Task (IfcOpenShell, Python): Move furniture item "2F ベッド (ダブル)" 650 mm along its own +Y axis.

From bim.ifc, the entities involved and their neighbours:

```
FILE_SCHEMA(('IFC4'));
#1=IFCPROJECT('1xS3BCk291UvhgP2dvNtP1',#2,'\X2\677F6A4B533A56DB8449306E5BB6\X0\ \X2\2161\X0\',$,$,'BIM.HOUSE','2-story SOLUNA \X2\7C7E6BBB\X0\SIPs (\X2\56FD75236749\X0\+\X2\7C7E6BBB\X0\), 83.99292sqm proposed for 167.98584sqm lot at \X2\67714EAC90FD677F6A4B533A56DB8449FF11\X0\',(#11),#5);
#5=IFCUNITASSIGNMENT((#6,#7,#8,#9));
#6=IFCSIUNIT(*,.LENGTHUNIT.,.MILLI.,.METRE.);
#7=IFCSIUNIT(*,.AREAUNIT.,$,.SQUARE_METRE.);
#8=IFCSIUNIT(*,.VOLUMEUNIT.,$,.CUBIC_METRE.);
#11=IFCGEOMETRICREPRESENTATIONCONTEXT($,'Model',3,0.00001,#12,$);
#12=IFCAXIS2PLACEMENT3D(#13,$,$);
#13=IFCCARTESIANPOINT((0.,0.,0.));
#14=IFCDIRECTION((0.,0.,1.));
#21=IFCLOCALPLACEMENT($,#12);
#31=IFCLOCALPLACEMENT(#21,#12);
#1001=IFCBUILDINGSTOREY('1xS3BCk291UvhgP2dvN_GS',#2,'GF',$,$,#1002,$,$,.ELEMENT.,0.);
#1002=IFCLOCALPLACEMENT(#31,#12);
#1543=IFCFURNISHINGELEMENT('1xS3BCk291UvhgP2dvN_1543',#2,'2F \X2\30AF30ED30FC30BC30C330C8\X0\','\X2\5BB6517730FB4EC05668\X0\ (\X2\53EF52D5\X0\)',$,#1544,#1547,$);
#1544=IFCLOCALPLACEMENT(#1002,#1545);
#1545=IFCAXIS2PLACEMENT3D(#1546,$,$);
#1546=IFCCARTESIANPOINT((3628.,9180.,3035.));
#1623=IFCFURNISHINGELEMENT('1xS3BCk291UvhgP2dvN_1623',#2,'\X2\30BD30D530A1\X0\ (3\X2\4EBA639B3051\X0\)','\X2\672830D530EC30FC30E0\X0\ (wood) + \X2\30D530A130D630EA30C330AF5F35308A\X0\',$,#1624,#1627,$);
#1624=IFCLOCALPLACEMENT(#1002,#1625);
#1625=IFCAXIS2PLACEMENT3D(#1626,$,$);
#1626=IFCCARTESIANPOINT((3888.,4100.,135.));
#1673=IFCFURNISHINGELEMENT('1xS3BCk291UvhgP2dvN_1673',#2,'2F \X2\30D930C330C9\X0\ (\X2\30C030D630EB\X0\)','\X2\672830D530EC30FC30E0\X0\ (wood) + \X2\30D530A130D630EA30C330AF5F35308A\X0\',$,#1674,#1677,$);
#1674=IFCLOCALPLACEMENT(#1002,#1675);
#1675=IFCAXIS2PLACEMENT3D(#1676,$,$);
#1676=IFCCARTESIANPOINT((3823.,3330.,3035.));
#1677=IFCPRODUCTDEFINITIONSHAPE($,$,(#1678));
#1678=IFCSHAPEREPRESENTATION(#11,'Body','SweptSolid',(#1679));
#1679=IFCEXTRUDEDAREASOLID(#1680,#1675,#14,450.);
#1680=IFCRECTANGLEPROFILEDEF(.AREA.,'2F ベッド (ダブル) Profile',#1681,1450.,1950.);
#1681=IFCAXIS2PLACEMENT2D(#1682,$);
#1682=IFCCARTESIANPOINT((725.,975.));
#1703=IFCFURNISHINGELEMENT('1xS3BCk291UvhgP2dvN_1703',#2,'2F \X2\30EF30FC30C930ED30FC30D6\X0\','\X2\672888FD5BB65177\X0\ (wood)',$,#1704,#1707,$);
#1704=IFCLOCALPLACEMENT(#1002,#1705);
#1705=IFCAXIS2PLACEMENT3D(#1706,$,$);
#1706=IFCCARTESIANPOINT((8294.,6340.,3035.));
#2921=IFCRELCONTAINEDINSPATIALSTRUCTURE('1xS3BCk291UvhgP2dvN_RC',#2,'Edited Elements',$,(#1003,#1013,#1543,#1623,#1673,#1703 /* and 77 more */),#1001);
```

```python
import ifcopenshell
import ifcopenshell.api.geometry
import ifcopenshell.util.placement

model = ifcopenshell.open("bim.ifc")

item = model.by_guid("1xS3BCk291UvhgP2dvN_1673")
matrix = ifcopenshell.util.placement.get_local_placement(item.ObjectPlacement)
matrix[:3, 3] += matrix[:3, 1] * 650.0
ifcopenshell.api.geometry.edit_object_placement(model, product=item, matrix=matrix, is_si=False)

print(ifcopenshell.util.placement.get_local_placement(item.ObjectPlacement).round(3) + 0.0)

model.write("bim_v2.ifc")
```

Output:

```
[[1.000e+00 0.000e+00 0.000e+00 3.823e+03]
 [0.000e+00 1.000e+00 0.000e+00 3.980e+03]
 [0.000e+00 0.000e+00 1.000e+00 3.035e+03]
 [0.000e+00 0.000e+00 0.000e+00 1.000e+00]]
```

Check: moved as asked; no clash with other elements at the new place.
